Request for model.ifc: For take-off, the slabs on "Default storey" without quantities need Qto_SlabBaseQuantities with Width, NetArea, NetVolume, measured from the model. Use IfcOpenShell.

First a look at what the model holds.

```python
import ifcopenshell
import ifcopenshell.util.element
import ifcopenshell.util.unit

model = ifcopenshell.open("model.ifc")
print(model.schema)
for unit_type in ("LENGTHUNIT", "AREAUNIT", "VOLUMEUNIT"):
    print(unit_type, ifcopenshell.util.unit.calculate_unit_scale(model, unit_type))
storey = next(s for s in model.by_type("IfcBuildingStorey") if s.Name == "Default storey")
slabs = [e for e in ifcopenshell.util.element.get_decomposition(storey) if e.is_a("IfcSlab")]
for e in sorted(slabs, key=lambda e: e.id()):
    print(e.id(), e.is_a(), e.Name, list(ifcopenshell.util.element.get_psets(e, qtos_only=True)), sep=" | ")
```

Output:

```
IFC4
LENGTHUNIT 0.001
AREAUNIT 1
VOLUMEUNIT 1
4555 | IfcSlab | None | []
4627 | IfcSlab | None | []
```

```python
import ifcopenshell
import ifcopenshell.api.pset
import ifcopenshell.geom
import ifcopenshell.util.element
import ifcopenshell.util.shape
import ifcopenshell.util.unit

model = ifcopenshell.open("model.ifc")
unit_scale = ifcopenshell.util.unit.calculate_unit_scale(model)
area_scale = ifcopenshell.util.unit.calculate_unit_scale(model, "AREAUNIT")
volume_scale = ifcopenshell.util.unit.calculate_unit_scale(model, "VOLUMEUNIT")
settings = ifcopenshell.geom.settings()

storey = next(s for s in model.by_type("IfcBuildingStorey") if s.Name == "Default storey")
slabs = [e for e in ifcopenshell.util.element.get_decomposition(storey) if e.is_a("IfcSlab")]

for e in sorted(slabs, key=lambda e: e.id()):
    if ifcopenshell.util.element.get_psets(e, qtos_only=True, should_inherit=False):
        continue
    # Geometry comes back in metres, in the element's own axes.
    shape = ifcopenshell.geom.create_shape(settings, e)
    values = {
        "Width": ifcopenshell.util.shape.get_z(shape.geometry) / unit_scale,
        "NetArea": ifcopenshell.util.shape.get_footprint_area(shape.geometry) / area_scale,
        "NetVolume": ifcopenshell.util.shape.get_volume(shape.geometry) / volume_scale,
    }
    qto = ifcopenshell.api.pset.add_qto(model, product=e, name="Qto_SlabBaseQuantities")
    ifcopenshell.api.pset.edit_qto(model, qto=qto, properties=values)
    print(e.id(), {k: round(v, 3) for k, v in values.items()})

model.write("model_updated.ifc")
```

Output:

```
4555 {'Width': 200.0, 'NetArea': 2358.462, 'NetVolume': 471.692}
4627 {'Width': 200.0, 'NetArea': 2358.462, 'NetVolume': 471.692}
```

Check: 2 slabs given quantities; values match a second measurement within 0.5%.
